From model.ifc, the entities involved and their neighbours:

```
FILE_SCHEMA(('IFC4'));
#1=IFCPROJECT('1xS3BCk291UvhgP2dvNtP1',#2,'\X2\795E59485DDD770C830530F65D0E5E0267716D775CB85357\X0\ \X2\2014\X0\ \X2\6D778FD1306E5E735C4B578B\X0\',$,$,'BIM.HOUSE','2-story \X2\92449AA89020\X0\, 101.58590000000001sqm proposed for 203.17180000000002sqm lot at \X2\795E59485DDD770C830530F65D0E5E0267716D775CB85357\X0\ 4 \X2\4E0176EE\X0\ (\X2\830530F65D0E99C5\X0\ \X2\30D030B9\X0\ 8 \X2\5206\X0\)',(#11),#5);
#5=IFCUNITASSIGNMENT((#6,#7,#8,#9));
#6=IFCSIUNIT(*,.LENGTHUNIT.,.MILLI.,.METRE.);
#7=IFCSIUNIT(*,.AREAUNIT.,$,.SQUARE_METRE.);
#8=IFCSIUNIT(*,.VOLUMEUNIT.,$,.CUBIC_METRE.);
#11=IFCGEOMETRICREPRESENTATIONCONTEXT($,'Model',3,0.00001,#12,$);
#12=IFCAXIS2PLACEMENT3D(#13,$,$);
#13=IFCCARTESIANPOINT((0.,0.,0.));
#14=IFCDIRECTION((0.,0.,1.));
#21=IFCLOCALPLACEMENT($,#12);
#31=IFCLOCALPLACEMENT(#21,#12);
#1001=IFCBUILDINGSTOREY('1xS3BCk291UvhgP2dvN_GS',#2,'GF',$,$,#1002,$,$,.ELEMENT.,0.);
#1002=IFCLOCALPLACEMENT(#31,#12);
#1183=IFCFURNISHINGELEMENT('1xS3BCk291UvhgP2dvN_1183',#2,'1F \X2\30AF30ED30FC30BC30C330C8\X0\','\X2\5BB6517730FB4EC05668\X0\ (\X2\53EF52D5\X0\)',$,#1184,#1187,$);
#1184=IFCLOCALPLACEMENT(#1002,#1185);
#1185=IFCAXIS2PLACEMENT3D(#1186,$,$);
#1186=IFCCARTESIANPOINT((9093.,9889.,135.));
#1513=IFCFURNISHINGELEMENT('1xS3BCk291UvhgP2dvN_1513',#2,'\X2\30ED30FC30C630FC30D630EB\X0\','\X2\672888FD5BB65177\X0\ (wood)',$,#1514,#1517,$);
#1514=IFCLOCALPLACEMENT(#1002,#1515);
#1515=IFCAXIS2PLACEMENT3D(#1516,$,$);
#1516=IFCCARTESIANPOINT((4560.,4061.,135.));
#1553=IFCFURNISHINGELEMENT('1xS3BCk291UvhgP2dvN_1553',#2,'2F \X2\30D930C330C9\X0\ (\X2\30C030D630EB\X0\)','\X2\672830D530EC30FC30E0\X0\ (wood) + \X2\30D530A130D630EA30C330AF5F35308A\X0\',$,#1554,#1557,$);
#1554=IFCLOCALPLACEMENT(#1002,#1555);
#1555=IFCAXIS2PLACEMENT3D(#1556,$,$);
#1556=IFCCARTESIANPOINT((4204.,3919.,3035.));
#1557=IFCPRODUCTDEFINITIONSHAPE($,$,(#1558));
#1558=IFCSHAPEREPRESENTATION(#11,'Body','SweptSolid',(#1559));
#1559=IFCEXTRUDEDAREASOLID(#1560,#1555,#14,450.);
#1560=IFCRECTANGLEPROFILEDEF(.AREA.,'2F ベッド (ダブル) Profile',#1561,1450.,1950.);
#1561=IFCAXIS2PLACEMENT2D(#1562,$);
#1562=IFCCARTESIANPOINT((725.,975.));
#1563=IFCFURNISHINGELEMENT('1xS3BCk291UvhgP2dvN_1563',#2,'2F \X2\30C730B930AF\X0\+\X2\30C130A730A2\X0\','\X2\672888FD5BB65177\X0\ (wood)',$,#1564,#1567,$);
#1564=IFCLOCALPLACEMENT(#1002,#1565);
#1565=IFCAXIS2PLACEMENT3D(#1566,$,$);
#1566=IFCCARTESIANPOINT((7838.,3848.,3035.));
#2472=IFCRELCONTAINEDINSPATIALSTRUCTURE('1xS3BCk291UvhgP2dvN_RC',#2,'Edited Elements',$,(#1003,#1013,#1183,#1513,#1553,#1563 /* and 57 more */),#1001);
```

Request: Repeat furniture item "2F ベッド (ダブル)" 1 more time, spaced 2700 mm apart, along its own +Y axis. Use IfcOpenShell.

```python
import ifcopenshell
import ifcopenshell.api.geometry
import ifcopenshell.api.root
import ifcopenshell.util.element
import ifcopenshell.util.placement
import ifcopenshell.util.unit

model = ifcopenshell.open("model.ifc")
unit_scale = ifcopenshell.util.unit.calculate_unit_scale(model)


def reuse_history(source, copy):
    """copy_class also copies each property set's owner history, people and application; keep the originals."""
    for rel in copy.IsDefinedBy:
        if rel.is_a("IfcRelDefinesByProperties") and (history := rel.RelatingPropertyDefinition.OwnerHistory):
            rel.RelatingPropertyDefinition.OwnerHistory = source.OwnerHistory
            ifcopenshell.util.element.remove_deep2(model, history)


source = model.by_id(1553)
base = ifcopenshell.util.placement.get_local_placement(source.ObjectPlacement)
step = base[:3, 1] * 2.7 / unit_scale

for i in range(1, 2):
    copy = ifcopenshell.api.root.copy_class(model, product=source)
    copy.Representation = ifcopenshell.util.element.copy_deep(
        model, source.Representation, exclude=["IfcGeometricRepresentationContext", "IfcRepresentationMap"]
    )
    reuse_history(source, copy)
    matrix = base.copy()
    matrix[:3, 3] += i * step
    print("added at", matrix[:3, 3].round(3) + 0.0)
    ifcopenshell.api.geometry.edit_object_placement(model, product=copy, matrix=matrix, is_si=False)

model.write("model_edited.ifc")
```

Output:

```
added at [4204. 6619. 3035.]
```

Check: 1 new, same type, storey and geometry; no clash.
